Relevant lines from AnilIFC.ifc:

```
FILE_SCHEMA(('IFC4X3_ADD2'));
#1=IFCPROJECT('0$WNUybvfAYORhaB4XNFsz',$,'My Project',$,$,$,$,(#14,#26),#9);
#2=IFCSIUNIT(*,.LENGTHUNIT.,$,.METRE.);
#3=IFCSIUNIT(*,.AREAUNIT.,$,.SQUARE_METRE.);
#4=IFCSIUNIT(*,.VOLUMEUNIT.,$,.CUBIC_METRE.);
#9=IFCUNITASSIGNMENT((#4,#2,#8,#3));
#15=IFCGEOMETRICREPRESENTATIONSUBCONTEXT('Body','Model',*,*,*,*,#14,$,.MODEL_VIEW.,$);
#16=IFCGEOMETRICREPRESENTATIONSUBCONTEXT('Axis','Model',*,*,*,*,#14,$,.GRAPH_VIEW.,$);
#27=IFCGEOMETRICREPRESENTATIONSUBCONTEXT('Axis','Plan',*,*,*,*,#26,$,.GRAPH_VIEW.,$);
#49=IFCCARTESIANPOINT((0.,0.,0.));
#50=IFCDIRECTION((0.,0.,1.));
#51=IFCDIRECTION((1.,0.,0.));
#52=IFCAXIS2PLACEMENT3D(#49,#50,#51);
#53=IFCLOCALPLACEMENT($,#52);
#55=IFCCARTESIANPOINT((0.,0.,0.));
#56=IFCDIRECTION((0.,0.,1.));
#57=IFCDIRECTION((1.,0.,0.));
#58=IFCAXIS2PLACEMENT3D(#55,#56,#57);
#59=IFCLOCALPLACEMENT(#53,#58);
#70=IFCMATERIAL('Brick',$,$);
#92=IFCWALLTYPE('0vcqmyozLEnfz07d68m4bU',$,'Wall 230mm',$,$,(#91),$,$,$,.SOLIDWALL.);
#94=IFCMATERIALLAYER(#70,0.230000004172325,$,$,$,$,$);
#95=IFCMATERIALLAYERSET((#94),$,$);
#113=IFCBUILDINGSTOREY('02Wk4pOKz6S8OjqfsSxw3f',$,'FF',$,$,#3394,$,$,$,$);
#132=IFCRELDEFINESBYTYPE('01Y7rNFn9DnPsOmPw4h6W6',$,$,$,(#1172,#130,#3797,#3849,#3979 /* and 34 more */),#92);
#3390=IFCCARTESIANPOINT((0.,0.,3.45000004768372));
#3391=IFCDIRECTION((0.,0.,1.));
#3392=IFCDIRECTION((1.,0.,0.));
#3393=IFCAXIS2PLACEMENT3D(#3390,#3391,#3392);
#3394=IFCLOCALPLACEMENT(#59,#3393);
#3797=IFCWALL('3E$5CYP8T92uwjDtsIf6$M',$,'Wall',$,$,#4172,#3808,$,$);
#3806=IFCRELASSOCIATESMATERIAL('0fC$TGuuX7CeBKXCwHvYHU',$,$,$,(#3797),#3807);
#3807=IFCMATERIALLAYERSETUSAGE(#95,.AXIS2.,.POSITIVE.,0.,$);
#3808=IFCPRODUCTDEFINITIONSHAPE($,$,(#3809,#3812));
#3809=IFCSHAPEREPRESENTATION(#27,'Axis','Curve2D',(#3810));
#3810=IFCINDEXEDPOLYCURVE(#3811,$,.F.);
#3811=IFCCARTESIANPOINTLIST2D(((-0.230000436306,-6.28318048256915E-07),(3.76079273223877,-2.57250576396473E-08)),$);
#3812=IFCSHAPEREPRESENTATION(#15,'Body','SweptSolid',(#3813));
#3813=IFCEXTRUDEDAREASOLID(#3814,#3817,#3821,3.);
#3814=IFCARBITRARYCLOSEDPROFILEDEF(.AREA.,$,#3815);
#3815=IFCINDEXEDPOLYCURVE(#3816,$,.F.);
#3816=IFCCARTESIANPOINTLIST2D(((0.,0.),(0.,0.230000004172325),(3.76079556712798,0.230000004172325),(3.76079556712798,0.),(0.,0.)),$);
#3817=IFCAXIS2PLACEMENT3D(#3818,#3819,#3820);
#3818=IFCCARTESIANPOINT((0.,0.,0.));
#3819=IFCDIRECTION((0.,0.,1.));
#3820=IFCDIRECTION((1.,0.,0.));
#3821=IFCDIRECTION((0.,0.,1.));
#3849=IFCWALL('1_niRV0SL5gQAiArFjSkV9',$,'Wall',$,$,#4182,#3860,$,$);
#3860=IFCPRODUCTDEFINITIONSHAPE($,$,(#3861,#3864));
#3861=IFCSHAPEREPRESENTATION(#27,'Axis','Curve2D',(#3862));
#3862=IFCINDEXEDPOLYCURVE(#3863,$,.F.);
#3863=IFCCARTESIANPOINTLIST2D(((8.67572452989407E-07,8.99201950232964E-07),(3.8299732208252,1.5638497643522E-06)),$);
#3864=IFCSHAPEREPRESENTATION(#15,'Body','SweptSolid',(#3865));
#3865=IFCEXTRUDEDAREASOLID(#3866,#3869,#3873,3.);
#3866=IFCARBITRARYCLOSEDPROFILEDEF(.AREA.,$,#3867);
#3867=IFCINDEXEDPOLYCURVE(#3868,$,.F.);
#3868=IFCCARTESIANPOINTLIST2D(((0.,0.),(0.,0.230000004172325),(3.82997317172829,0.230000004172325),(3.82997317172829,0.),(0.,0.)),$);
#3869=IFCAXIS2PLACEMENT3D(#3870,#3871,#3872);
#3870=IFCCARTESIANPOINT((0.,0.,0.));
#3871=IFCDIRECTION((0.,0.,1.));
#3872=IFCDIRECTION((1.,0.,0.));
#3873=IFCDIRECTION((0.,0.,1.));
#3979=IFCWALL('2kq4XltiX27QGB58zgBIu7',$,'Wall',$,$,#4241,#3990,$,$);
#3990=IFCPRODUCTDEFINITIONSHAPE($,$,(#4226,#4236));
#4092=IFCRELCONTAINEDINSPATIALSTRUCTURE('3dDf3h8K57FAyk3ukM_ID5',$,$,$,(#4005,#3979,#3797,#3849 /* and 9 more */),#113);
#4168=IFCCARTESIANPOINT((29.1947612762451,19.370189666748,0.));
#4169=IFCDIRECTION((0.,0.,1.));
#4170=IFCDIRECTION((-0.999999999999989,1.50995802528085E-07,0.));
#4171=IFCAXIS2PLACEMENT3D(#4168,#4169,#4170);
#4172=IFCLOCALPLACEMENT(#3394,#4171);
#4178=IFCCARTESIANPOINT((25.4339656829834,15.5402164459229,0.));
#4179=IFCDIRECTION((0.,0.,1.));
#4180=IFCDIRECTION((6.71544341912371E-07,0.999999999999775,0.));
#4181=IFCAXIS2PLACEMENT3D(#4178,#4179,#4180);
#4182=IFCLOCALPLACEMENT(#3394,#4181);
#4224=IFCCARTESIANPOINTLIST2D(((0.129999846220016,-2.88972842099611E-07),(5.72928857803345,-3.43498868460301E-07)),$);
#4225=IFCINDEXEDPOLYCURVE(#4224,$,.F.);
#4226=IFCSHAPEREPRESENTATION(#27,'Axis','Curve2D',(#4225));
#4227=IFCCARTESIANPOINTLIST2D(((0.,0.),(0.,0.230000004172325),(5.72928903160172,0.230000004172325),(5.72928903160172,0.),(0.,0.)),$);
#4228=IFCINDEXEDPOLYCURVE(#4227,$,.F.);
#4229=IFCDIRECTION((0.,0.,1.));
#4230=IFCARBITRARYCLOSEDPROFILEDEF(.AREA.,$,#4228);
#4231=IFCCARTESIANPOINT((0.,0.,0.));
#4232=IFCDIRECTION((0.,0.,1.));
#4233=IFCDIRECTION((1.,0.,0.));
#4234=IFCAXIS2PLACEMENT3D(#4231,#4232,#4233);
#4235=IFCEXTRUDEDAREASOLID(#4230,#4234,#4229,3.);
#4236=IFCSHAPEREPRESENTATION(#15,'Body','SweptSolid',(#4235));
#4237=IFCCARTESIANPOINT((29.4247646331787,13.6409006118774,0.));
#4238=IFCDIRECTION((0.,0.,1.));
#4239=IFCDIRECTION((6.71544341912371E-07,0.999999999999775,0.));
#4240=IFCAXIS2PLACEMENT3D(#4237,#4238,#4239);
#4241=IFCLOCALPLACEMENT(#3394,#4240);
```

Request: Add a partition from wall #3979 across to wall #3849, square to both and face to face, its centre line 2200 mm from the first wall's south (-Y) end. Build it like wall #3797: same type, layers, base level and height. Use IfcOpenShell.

```python
import numpy as np
import ifcopenshell
import ifcopenshell.api.geometry
import ifcopenshell.api.material
import ifcopenshell.api.pset
import ifcopenshell.api.root
import ifcopenshell.api.spatial
import ifcopenshell.api.type
import ifcopenshell.geom
import ifcopenshell.util.element
import ifcopenshell.util.placement
import ifcopenshell.util.representation
import ifcopenshell.util.shape
import ifcopenshell.util.unit

model = ifcopenshell.open("AnilIFC.ifc")
unit_scale = ifcopenshell.util.unit.calculate_unit_scale(model)
settings = ifcopenshell.geom.settings()
settings.set("use-world-coords", True)

start_wall = model.by_guid("2kq4XltiX27QGB58zgBIu7")
end_wall = model.by_guid("1_niRV0SL5gQAiArFjSkV9")
like = model.by_guid("3E$5CYP8T92uwjDtsIf6$M")
matrix = ifcopenshell.util.placement.get_local_placement(start_wall.ObjectPlacement)
matrix[:3, 3] *= unit_scale


def extent(element):
    """Bounding box in the first wall's axes, in metres."""
    shape = ifcopenshell.geom.create_shape(settings, element)
    points = (ifcopenshell.util.shape.get_vertices(shape.geometry) - matrix[:3, 3]) @ matrix[:3, :3]
    return points.min(axis=0), points.max(axis=0)


y_start = extent(start_wall)[1][1]
y_end = extent(end_wall)[0][1]
like_min, like_max = extent(like)
length, height = float(abs(y_end - y_start)), float(like_max[2] - like_min[2])
layer_set = ifcopenshell.util.element.get_material(like, should_skip_usage=True)
thickness = sum(layer.LayerThickness for layer in layer_set.MaterialLayers) * unit_scale

wall = ifcopenshell.api.root.create_entity(model, ifc_class="IfcWall", name="New partition")
storey = ifcopenshell.util.element.get_container(like)
ifcopenshell.api.spatial.assign_container(model, products=[wall], relating_structure=storey)
ifcopenshell.api.type.assign_type(
    model, related_objects=[wall], relating_type=ifcopenshell.util.element.get_type(like), should_map_representations=False
)
rel = ifcopenshell.api.material.assign_material(
    model, products=[wall], type="IfcMaterialLayerSetUsage", material=layer_set
)
rel.RelatingMaterial.OffsetFromReferenceLine = -thickness / 2 / unit_scale
pset = ifcopenshell.api.pset.add_pset(model, product=wall, name="Pset_WallCommon")
ifcopenshell.api.pset.edit_pset(model, pset=pset, properties={"IsExternal": False, "LoadBearing": False})

# The axis runs down the middle of the wall.
axis = ifcopenshell.api.geometry.add_axis_representation(
    model, context=ifcopenshell.util.representation.get_context(model, "Model", "Axis"), axis=[(0.0, 0.0), (length, 0.0)]
)
body = ifcopenshell.api.geometry.add_wall_representation(
    model,
    context=ifcopenshell.util.representation.get_context(model, "Model", "Body", "MODEL_VIEW"),
    length=length,
    height=height,
    thickness=thickness,
    offset=-thickness / 2,
)
for representation in (axis, body):
    ifcopenshell.api.geometry.assign_representation(model, product=wall, representation=representation)

placement = matrix @ ifcopenshell.util.placement.rotation(90, "Z")
placement[:, 3] = matrix @ np.array([extent(start_wall)[0][0] + 2.2, y_start, like_min[2], 1.0])
ifcopenshell.api.geometry.edit_object_placement(model, product=wall, matrix=placement)

print(f"partition {length:.3f} m long, {height:.3f} m high, {thickness:.3f} m thick")

model.write("AnilIFC_updated.ifc")
```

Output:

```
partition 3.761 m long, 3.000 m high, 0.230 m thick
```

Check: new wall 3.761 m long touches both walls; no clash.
